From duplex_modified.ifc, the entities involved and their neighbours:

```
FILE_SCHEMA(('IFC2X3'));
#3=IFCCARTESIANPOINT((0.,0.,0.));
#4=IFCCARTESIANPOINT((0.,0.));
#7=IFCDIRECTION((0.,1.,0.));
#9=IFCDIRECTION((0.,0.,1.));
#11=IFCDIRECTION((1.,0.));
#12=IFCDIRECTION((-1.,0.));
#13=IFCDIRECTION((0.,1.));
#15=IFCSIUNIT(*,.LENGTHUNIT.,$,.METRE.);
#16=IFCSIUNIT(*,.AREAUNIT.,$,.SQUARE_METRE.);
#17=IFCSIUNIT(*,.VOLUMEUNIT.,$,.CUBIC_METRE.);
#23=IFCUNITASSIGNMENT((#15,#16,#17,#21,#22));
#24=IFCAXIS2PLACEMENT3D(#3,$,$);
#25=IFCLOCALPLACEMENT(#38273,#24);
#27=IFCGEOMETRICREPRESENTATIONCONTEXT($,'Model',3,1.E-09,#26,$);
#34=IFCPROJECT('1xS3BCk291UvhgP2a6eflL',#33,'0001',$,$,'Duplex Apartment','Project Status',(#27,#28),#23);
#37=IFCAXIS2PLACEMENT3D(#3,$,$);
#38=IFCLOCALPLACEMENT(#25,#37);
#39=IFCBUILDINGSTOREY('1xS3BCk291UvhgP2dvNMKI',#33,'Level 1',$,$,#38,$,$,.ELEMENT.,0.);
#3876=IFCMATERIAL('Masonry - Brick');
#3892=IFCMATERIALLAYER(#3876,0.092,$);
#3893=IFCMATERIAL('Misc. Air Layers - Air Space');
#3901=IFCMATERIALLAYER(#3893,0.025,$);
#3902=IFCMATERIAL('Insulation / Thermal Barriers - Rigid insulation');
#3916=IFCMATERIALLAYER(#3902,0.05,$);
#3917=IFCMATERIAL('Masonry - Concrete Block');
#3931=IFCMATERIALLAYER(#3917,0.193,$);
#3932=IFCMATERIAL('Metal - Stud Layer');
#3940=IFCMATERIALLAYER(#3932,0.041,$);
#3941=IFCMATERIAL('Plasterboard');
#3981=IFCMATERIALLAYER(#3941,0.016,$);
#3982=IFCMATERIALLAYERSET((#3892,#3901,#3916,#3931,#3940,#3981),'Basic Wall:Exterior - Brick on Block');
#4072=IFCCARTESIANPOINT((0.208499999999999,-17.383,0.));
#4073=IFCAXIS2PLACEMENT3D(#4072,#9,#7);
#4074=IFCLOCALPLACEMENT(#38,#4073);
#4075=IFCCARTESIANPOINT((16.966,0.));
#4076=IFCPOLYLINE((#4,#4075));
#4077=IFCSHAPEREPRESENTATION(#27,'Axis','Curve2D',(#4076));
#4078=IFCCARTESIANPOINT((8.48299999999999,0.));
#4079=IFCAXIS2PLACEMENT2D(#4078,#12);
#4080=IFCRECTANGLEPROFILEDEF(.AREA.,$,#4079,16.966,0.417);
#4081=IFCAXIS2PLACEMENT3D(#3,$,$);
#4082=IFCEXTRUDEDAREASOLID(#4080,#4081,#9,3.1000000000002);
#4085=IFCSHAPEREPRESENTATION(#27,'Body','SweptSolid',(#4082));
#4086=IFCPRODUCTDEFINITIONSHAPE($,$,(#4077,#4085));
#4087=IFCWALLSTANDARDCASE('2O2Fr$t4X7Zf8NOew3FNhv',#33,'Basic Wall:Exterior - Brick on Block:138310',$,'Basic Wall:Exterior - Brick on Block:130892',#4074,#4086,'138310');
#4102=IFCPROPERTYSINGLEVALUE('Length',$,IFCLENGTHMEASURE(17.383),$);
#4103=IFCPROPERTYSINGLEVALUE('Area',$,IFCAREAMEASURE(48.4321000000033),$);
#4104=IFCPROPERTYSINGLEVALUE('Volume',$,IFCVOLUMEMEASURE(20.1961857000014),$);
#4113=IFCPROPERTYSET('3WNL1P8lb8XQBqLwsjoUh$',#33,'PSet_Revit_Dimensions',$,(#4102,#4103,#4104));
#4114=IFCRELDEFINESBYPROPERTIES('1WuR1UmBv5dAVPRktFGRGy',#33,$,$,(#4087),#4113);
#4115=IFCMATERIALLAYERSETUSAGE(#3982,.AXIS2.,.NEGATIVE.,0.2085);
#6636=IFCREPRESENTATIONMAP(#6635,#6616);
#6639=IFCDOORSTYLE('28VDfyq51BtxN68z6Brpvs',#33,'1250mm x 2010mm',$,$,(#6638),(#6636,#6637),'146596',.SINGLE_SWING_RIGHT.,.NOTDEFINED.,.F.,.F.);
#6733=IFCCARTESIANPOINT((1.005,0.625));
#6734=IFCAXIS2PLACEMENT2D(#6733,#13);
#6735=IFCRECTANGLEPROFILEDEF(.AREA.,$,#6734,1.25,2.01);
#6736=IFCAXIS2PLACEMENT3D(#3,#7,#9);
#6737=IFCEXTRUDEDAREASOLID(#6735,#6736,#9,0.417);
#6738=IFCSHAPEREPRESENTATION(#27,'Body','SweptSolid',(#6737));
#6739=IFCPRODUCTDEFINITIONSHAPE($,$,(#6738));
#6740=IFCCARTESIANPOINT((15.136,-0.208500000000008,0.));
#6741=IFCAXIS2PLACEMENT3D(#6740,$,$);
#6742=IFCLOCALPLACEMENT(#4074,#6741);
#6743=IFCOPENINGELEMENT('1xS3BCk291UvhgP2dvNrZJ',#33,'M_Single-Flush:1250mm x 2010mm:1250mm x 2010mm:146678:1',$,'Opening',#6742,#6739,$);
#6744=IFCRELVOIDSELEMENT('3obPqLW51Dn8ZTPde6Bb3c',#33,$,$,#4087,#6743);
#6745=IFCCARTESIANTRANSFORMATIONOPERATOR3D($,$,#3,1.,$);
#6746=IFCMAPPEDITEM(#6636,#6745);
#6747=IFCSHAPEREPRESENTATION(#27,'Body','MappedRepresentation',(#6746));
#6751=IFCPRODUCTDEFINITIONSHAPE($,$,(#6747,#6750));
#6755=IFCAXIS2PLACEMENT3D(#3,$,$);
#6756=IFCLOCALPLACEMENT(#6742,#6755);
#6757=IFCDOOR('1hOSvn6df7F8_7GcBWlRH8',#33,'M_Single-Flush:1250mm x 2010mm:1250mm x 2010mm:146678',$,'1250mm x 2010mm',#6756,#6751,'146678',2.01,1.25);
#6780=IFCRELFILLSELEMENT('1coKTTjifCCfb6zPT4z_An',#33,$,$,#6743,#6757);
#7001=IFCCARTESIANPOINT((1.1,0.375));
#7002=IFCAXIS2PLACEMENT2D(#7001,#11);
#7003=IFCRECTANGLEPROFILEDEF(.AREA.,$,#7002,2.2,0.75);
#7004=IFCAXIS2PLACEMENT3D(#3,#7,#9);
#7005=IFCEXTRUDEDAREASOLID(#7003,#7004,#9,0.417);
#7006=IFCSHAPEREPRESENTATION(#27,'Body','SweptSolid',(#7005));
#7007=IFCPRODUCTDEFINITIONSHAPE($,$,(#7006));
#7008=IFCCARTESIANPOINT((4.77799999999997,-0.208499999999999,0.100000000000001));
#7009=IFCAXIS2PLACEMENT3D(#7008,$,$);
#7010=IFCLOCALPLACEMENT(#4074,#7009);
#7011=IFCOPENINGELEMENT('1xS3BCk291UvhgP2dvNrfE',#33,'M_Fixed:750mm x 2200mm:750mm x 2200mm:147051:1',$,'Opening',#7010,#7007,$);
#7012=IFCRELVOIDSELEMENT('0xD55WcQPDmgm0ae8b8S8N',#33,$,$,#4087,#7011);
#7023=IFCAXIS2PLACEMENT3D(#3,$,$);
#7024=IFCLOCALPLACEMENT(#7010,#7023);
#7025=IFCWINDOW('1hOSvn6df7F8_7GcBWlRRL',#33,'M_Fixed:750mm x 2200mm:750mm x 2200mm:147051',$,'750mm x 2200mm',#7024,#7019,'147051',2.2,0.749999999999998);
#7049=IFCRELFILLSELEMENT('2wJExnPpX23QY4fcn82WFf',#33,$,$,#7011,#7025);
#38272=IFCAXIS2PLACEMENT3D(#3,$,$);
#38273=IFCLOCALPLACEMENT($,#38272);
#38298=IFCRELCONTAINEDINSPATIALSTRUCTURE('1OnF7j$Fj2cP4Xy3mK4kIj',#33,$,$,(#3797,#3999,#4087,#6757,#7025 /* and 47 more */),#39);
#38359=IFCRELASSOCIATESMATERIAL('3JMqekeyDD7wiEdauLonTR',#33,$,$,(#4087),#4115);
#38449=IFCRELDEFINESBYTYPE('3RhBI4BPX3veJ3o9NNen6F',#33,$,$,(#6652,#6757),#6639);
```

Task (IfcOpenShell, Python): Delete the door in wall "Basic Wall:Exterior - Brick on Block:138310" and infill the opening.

```python
import ifcopenshell
import ifcopenshell.api.feature
import ifcopenshell.api.pset
import ifcopenshell.api.root
import ifcopenshell.geom
import ifcopenshell.util.element
import ifcopenshell.util.shape
import ifcopenshell.util.unit

model = ifcopenshell.open("duplex_modified.ifc")
area_scale = ifcopenshell.util.unit.calculate_unit_scale(model, "AREAUNIT")
volume_scale = ifcopenshell.util.unit.calculate_unit_scale(model, "VOLUMEUNIT")
settings = ifcopenshell.geom.settings()


def volume(element):
    """Net volume in cubic metres, openings subtracted."""
    shape = ifcopenshell.geom.create_shape(settings, element)
    return ifcopenshell.util.shape.get_volume(shape.geometry)


door = model.by_guid("1hOSvn6df7F8_7GcBWlRH8")
opening = door.FillsVoids[0].RelatingOpeningElement
wall = opening.VoidsElements[0].RelatingBuildingElement
before = volume(wall)

ifcopenshell.api.root.remove_product(model, product=door)
ifcopenshell.api.feature.remove_feature(model, feature=opening)

after = volume(wall)
thickness = 0.417  # wall thickness in metres

# Update the wall's stored quantities.
pset = model.by_id(ifcopenshell.util.element.get_pset(wall, "PSet_Revit_Dimensions", should_inherit=False)["id"])
ifcopenshell.api.pset.edit_pset(model, pset=pset, properties={
    "Area": model.create_entity("IfcAreaMeasure", after / thickness / area_scale),
    "Volume": model.create_entity("IfcVolumeMeasure", after / volume_scale),
})

print(f"wall volume {before:.3f} -> {after:.3f} m3")

model.write("duplex_modified-out.ifc")
```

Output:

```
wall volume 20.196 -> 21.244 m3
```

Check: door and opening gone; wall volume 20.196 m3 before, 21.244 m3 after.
